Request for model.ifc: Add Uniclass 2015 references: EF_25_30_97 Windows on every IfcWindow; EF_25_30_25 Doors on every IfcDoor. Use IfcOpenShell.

First a look at what the model holds.

```python
import ifcopenshell

model = ifcopenshell.open("model.ifc")
print(model.schema)
print("classifications:", [c.Name for c in model.by_type("IfcClassification")])
for ifc_class in ("IfcDoor", "IfcRoof", "IfcStair", "IfcWall", "IfcWindow"):
    print(ifc_class, len(model.by_type(ifc_class)))
```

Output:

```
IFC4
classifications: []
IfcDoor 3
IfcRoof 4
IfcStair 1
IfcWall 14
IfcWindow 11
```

```python
import ifcopenshell
import ifcopenshell.api.classification

model = ifcopenshell.open("model.ifc")

system = ifcopenshell.api.classification.add_classification(model, classification="Uniclass 2015")

codes = {
    "IfcWindow": ("EF_25_30_97", "Windows"),
    "IfcDoor": ("EF_25_30_25", "Doors"),
}
for ifc_class, (code, name) in codes.items():
    products = model.by_type(ifc_class)
    ifcopenshell.api.classification.add_reference(
        model, products=products, classification=system, identification=code, name=name
    )
    print(code, len(products))

model.write("model-out.ifc")
```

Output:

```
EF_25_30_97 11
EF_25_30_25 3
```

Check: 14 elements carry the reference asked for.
